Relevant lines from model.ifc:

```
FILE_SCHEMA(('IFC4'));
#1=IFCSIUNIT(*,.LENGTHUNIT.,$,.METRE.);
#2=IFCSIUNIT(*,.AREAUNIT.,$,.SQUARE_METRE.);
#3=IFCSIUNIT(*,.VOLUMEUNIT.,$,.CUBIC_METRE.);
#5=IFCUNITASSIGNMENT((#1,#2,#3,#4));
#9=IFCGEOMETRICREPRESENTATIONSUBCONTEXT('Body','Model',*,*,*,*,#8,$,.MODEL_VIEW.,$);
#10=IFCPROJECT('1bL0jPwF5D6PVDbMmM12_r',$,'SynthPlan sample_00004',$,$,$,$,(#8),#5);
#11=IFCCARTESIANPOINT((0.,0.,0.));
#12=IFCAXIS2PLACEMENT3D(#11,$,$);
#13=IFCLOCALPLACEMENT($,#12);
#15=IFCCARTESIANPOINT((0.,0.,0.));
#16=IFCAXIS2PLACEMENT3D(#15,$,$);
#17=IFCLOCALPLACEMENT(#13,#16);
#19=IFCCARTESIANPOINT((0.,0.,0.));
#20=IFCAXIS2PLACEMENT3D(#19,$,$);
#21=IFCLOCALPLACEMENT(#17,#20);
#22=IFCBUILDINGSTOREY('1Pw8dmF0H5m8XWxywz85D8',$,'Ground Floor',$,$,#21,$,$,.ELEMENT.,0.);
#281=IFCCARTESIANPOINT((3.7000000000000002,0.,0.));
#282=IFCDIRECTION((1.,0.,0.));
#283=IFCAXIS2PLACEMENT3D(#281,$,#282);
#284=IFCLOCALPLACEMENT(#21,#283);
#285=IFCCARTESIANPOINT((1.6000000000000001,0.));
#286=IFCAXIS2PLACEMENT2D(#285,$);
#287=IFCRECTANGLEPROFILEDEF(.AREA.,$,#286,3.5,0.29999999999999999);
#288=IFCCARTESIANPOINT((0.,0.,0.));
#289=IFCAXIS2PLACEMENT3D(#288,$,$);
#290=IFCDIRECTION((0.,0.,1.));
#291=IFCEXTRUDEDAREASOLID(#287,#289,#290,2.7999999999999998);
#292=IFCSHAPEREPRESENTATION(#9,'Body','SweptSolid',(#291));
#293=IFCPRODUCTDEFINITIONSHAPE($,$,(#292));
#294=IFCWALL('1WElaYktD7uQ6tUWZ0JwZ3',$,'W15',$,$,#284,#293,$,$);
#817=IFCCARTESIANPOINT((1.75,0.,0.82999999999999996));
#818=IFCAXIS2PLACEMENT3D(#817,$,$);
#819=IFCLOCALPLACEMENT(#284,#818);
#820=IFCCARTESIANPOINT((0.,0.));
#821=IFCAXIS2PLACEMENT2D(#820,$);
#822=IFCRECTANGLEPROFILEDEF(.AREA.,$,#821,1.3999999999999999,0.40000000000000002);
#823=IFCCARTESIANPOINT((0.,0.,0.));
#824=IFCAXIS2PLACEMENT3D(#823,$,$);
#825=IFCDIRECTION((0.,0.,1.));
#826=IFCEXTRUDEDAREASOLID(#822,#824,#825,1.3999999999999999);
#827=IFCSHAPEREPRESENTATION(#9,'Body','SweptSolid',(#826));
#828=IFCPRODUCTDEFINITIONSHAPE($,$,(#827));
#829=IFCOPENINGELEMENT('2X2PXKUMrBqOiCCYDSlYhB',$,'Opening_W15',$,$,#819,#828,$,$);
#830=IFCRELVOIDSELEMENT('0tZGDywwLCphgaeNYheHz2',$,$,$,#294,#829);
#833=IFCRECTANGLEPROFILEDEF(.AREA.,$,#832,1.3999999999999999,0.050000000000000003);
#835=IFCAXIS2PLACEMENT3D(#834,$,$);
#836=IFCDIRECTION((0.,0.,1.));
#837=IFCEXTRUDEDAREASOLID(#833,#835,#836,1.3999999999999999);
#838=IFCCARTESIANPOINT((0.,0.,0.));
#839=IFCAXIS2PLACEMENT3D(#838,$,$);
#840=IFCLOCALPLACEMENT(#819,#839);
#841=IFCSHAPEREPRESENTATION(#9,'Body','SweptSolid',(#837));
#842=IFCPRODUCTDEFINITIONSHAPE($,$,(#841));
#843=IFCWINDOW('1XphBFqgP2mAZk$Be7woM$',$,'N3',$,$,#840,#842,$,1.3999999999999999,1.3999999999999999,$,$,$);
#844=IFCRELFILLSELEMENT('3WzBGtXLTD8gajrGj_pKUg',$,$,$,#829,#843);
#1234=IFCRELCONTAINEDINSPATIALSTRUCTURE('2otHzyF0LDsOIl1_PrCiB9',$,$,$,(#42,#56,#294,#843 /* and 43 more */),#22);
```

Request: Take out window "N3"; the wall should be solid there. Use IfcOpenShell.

```python
import ifcopenshell
import ifcopenshell.api.feature
import ifcopenshell.api.root
import ifcopenshell.geom
import ifcopenshell.util.shape

model = ifcopenshell.open("model.ifc")
settings = ifcopenshell.geom.settings()


def volume(element):
    """Net volume in cubic metres, openings subtracted."""
    shape = ifcopenshell.geom.create_shape(settings, element)
    return ifcopenshell.util.shape.get_volume(shape.geometry)


window = model.by_id(843)
opening = window.FillsVoids[0].RelatingOpeningElement
wall = opening.VoidsElements[0].RelatingBuildingElement
before = volume(wall)

ifcopenshell.api.root.remove_product(model, product=window)
ifcopenshell.api.feature.remove_feature(model, feature=opening)

after = volume(wall)

print(f"wall volume {before:.3f} -> {after:.3f} m3")

model.write("model_edited.ifc")
```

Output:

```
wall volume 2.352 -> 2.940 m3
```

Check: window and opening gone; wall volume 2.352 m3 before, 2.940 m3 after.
